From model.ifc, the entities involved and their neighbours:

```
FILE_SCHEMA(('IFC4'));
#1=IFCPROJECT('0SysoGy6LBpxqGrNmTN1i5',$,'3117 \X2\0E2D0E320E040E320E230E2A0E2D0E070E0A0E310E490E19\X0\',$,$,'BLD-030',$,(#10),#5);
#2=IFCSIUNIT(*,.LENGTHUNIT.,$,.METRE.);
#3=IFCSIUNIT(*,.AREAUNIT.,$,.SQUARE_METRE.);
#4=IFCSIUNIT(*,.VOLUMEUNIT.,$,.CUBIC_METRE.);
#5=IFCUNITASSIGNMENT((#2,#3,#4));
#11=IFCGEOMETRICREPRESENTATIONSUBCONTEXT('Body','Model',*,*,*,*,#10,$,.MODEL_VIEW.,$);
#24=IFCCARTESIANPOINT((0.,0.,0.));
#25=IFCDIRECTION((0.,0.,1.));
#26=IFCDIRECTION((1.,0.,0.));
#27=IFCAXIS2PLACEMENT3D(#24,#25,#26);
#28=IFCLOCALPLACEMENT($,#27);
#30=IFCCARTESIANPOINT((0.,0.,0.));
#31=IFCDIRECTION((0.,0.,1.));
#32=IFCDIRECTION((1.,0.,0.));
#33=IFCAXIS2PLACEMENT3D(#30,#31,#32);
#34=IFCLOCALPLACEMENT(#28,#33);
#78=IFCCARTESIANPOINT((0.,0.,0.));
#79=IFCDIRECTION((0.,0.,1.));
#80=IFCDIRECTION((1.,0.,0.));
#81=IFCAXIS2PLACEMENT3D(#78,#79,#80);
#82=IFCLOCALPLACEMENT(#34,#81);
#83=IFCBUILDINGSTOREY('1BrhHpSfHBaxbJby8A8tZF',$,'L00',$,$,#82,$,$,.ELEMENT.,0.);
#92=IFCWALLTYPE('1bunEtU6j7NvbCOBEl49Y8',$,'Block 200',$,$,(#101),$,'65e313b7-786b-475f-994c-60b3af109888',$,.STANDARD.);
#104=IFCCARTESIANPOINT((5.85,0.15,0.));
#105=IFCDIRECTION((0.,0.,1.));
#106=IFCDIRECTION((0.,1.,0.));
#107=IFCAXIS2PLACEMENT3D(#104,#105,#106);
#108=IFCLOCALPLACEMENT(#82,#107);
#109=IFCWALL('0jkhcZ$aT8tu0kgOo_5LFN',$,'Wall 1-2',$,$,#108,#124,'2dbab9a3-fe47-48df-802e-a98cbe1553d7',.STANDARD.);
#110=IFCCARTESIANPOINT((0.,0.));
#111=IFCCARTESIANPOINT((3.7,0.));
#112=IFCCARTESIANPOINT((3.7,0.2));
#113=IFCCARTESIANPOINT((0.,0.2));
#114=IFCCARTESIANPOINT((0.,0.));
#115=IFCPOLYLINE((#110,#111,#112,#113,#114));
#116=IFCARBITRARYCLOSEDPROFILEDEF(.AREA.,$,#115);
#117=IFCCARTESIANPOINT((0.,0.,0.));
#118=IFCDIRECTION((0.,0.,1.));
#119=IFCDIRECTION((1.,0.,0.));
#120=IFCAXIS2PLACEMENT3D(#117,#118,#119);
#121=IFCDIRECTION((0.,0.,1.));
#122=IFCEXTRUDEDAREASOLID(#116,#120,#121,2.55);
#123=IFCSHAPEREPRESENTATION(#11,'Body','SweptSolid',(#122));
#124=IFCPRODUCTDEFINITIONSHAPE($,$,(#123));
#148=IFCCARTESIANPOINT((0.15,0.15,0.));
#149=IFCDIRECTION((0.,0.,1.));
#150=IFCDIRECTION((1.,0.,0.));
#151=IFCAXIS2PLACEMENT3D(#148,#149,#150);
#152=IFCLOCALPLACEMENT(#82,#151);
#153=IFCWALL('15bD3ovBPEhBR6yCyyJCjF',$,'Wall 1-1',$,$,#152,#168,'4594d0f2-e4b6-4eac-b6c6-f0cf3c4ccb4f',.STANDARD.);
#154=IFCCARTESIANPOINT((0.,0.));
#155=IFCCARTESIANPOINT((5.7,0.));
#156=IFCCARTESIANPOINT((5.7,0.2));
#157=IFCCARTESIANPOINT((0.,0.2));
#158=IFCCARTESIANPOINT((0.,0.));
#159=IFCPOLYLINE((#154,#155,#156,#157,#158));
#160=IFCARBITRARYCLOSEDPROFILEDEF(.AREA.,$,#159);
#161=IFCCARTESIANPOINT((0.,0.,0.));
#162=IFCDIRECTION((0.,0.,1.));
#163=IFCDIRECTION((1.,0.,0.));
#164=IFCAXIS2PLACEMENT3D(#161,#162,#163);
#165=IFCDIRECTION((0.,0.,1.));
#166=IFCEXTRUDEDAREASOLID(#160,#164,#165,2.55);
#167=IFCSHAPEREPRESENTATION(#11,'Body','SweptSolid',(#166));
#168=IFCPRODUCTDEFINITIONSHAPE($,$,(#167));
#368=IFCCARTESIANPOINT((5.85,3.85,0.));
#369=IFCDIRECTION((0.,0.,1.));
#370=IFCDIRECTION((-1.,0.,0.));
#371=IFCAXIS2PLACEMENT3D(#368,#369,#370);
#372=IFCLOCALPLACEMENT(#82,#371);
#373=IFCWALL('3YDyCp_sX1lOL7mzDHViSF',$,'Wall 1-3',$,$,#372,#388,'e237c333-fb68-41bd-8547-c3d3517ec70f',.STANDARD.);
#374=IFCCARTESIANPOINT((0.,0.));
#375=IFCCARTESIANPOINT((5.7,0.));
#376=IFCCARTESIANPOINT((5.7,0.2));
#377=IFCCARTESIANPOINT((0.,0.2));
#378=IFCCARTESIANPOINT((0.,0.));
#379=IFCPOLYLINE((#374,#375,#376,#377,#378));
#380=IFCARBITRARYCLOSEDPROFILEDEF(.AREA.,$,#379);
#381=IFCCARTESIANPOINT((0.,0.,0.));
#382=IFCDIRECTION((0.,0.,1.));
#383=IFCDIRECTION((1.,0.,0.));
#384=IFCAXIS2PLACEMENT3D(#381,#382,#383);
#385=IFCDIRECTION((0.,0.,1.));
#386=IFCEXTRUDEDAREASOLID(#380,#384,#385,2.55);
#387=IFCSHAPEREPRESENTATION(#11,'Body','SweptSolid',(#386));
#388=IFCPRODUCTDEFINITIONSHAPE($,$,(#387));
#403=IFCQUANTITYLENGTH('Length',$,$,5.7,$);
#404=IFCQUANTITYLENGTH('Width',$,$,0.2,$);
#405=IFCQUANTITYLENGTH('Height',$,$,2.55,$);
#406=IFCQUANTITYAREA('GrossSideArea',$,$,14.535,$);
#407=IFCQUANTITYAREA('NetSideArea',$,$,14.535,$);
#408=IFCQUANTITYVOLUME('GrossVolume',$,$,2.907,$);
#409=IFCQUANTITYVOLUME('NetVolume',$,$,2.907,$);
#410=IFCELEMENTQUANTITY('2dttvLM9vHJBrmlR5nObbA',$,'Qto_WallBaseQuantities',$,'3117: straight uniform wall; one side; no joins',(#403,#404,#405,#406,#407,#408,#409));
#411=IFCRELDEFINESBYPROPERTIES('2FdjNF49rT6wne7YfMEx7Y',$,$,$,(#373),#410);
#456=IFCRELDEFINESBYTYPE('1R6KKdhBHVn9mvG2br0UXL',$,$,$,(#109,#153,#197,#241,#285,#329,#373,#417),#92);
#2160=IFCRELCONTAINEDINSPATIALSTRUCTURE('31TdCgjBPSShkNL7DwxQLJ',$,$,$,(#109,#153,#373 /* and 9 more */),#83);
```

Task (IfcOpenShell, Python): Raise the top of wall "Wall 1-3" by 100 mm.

```python
import ifcopenshell
import ifcopenshell.api.pset
import ifcopenshell.geom
import ifcopenshell.util.element
import ifcopenshell.util.representation
import ifcopenshell.util.shape
import ifcopenshell.util.unit

model = ifcopenshell.open("model.ifc")
unit_scale = ifcopenshell.util.unit.calculate_unit_scale(model)
area_scale = ifcopenshell.util.unit.calculate_unit_scale(model, "AREAUNIT")
volume_scale = ifcopenshell.util.unit.calculate_unit_scale(model, "VOLUMEUNIT")
settings = ifcopenshell.geom.settings()


def volume(element):
    """Net volume in cubic metres, openings subtracted."""
    shape = ifcopenshell.geom.create_shape(settings, element)
    return ifcopenshell.util.shape.get_volume(shape.geometry)


wall = model.by_guid("3YDyCp_sX1lOL7mzDHViSF")
before = volume(wall)

body = ifcopenshell.util.representation.get_representation(wall, "Model", "Body")
solid = body.Items[0]
old_height = solid.Depth
solid.Depth += 0.1
after = volume(wall)
thickness = 0.2  # wall thickness in metres

# Update the stored height, areas and volumes.
qto = model.by_id(ifcopenshell.util.element.get_pset(wall, "Qto_WallBaseQuantities", should_inherit=False)["id"])
ifcopenshell.api.pset.edit_qto(model, qto=qto, properties={
    "Height": solid.Depth,
    "GrossSideArea": ifcopenshell.util.element.get_pset(wall, "Qto_WallBaseQuantities", "GrossSideArea") * solid.Depth / old_height,
    "NetSideArea": after / thickness / area_scale,
    "GrossVolume": ifcopenshell.util.element.get_pset(wall, "Qto_WallBaseQuantities", "GrossVolume") * solid.Depth / old_height,
    "NetVolume": after / volume_scale,
})

print(f"height {old_height:g} -> {solid.Depth:g}, volume {before:.3f} -> {after:.3f} m3")

model.write("model_v2.ifc")
```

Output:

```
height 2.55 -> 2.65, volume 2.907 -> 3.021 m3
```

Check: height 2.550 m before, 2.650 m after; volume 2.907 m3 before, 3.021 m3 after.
